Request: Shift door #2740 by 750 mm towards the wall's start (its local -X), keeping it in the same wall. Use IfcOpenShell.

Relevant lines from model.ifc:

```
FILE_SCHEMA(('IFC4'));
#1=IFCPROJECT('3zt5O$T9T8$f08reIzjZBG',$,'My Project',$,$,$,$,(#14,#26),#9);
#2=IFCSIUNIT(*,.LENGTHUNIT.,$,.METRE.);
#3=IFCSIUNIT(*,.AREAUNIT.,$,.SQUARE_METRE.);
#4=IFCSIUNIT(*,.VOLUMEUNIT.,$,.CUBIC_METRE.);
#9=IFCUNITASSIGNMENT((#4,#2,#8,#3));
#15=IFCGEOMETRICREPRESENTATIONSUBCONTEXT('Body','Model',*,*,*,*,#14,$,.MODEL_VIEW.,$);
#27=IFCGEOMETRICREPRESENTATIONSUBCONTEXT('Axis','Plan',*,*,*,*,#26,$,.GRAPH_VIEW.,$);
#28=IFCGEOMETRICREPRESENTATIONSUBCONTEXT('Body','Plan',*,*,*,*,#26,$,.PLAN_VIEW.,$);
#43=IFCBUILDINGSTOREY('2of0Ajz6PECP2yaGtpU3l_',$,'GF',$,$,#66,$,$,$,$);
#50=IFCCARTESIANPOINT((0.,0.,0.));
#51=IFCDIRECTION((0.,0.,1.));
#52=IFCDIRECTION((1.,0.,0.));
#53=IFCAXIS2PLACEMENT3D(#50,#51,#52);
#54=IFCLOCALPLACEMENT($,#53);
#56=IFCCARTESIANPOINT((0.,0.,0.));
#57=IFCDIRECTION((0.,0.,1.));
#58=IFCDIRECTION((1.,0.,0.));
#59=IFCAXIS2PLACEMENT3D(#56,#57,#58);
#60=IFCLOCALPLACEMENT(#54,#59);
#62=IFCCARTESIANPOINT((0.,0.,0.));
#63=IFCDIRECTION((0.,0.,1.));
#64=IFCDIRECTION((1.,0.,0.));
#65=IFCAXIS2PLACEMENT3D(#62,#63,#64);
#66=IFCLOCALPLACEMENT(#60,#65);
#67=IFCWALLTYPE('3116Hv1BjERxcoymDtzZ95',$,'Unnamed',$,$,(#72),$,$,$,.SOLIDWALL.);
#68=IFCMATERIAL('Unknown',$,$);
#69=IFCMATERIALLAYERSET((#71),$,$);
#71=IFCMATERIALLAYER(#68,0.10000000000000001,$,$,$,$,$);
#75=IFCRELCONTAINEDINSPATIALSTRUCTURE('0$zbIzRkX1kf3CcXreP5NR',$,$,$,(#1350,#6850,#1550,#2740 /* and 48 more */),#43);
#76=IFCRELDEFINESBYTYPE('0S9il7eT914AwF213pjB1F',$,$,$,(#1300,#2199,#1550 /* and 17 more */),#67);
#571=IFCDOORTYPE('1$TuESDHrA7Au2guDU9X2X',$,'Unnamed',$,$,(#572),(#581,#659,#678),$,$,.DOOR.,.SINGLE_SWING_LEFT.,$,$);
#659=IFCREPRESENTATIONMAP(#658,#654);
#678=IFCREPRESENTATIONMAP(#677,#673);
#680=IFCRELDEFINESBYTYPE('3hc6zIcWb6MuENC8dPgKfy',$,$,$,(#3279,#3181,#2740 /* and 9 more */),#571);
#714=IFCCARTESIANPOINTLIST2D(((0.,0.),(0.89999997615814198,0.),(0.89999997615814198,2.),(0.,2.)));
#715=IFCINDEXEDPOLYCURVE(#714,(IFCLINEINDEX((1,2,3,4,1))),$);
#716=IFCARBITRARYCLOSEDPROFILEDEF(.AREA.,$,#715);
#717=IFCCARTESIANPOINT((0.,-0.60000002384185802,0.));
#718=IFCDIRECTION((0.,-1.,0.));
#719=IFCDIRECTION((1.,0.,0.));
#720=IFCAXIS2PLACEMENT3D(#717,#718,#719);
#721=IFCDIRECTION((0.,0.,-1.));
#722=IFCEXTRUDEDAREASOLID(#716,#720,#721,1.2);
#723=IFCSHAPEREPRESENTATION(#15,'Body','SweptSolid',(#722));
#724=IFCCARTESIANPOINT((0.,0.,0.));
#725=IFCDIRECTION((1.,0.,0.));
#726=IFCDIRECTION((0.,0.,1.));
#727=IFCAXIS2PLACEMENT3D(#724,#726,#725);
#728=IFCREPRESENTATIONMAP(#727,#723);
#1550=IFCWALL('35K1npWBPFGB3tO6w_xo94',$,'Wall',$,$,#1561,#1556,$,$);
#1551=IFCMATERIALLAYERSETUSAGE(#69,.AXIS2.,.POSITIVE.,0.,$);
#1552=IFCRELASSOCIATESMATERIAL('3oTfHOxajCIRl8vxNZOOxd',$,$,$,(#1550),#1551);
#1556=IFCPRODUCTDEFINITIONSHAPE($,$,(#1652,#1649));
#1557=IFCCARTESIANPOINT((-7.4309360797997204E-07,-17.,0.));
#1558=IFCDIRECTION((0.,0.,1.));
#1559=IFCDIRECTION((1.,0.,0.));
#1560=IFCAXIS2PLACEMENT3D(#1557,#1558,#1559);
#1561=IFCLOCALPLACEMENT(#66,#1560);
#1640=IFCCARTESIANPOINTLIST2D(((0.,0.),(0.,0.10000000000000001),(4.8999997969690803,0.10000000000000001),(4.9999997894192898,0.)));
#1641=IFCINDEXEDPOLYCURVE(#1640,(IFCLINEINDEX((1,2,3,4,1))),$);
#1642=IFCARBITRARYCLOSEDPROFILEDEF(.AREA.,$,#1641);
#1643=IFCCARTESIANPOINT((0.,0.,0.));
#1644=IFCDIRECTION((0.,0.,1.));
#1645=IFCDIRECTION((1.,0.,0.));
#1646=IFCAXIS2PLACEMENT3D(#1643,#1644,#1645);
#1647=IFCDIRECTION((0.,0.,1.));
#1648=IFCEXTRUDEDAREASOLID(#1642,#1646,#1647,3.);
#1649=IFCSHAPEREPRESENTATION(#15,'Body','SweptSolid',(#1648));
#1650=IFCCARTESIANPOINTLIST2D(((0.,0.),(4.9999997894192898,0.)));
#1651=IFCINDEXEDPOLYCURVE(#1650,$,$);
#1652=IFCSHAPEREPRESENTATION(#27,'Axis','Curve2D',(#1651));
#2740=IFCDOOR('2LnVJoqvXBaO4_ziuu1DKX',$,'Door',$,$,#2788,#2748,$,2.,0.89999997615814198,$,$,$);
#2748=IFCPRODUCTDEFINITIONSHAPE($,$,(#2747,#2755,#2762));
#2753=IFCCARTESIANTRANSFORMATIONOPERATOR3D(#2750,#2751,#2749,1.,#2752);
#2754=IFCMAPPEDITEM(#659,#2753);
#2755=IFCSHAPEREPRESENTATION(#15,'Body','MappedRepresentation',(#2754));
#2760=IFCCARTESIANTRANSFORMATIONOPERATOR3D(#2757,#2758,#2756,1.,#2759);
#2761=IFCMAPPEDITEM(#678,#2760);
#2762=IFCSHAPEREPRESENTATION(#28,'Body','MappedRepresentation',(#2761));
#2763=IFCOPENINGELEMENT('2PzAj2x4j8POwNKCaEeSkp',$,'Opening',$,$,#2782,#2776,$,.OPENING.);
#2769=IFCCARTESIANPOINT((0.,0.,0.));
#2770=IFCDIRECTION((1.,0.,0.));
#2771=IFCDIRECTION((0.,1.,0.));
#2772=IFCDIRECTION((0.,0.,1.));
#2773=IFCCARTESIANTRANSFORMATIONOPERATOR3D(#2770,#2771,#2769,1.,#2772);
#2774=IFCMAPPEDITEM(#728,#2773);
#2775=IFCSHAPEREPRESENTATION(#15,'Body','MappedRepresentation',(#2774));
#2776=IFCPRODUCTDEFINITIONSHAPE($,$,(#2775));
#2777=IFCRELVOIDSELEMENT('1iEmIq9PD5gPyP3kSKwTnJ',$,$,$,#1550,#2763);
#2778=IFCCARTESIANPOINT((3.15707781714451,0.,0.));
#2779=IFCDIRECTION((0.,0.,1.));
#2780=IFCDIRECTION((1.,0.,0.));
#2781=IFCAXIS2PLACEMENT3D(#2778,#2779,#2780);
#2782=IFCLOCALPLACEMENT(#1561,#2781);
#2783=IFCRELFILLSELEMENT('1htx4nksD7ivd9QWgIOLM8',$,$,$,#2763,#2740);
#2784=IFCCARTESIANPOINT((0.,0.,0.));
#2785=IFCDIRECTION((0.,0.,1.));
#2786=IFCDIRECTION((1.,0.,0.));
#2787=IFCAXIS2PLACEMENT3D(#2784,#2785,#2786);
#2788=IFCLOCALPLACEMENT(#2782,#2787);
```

```python
import ifcopenshell
import ifcopenshell.api.geometry
import ifcopenshell.util.placement
import ifcopenshell.util.unit

model = ifcopenshell.open("model.ifc")
unit_scale = ifcopenshell.util.unit.calculate_unit_scale(model)

door = model.by_guid("2LnVJoqvXBaO4_ziuu1DKX")
opening = door.FillsVoids[0].RelatingOpeningElement
wall = opening.VoidsElements[0].RelatingBuildingElement

wall_matrix = ifcopenshell.util.placement.get_local_placement(wall.ObjectPlacement)
shift = wall_matrix[:3, 0] * -0.75 / unit_scale
before = ifcopenshell.util.placement.get_local_placement(door.ObjectPlacement)[:3, 3].copy()

# The door is placed relative to its opening, so it follows when the opening moves.
matrix = ifcopenshell.util.placement.get_local_placement(opening.ObjectPlacement)
matrix[:3, 3] += shift
ifcopenshell.api.geometry.edit_object_placement(
    model, product=opening, matrix=matrix, is_si=False, should_transform_children=True
)

after = ifcopenshell.util.placement.get_local_placement(door.ObjectPlacement)[:3, 3]
print("door moved by", (after - before).round(3) + 0.0)

model.write("model_rev.ifc")
```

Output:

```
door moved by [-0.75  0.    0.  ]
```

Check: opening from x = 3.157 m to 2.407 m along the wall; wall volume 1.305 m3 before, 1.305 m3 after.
